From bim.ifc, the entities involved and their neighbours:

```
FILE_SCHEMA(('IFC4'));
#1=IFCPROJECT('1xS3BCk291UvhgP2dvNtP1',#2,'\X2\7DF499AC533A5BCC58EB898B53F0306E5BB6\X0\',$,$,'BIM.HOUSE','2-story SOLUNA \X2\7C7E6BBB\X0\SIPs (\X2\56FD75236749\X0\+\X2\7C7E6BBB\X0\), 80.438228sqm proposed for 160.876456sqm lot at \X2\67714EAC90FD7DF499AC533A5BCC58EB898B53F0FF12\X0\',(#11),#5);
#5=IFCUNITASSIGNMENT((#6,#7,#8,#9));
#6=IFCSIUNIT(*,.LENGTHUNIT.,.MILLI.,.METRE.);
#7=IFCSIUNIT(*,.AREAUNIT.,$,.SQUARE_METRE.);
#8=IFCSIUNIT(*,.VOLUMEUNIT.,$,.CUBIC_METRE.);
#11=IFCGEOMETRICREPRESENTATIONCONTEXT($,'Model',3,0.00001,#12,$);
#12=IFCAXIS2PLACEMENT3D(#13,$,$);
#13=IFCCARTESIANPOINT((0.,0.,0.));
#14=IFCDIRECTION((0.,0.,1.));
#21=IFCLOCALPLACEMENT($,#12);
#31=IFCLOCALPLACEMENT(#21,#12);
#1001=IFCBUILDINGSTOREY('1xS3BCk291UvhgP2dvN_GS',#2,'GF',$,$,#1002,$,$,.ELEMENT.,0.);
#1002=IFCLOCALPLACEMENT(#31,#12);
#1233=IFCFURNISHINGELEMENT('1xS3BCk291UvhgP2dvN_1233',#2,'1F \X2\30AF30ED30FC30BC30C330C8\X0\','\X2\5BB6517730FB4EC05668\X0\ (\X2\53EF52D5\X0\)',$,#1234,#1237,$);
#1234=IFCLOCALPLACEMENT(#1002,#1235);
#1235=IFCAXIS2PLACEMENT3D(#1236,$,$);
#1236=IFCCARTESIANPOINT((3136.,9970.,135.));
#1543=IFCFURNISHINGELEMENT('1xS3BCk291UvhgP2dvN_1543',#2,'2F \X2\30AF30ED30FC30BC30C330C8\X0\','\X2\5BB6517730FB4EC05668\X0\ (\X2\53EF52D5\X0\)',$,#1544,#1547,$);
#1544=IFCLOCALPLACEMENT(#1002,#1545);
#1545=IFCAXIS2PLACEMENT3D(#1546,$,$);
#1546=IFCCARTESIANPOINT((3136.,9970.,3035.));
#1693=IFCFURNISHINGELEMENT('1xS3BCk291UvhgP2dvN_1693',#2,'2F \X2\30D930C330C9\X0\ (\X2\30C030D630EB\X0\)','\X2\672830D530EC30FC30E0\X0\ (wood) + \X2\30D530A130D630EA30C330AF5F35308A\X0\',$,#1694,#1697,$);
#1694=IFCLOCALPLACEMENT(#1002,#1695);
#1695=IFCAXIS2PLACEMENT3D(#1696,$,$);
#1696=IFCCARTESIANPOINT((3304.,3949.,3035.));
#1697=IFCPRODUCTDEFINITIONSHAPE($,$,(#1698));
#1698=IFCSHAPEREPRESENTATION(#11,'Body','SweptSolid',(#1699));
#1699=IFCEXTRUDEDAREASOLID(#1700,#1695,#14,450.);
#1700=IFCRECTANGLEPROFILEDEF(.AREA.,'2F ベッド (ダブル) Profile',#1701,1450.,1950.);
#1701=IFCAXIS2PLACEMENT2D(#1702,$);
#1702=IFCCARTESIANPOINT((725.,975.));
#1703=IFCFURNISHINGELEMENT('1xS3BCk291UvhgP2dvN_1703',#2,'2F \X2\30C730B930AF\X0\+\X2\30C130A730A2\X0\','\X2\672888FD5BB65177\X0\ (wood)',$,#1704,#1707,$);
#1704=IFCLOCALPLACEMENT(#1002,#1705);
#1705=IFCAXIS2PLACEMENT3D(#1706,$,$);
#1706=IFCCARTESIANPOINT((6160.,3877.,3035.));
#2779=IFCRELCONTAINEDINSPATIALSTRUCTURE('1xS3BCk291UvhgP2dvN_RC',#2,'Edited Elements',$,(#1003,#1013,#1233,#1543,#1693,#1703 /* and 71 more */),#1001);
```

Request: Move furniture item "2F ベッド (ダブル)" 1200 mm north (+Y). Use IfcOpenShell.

```python
import ifcopenshell
import ifcopenshell.api.geometry
import ifcopenshell.util.placement

model = ifcopenshell.open("bim.ifc")

item = model.by_id(1693)
matrix = ifcopenshell.util.placement.get_local_placement(item.ObjectPlacement)
matrix[1, 3] += 1200.0
ifcopenshell.api.geometry.edit_object_placement(model, product=item, matrix=matrix, is_si=False)

print(ifcopenshell.util.placement.get_local_placement(item.ObjectPlacement).round(3) + 0.0)

model.write("bim_rev.ifc")
```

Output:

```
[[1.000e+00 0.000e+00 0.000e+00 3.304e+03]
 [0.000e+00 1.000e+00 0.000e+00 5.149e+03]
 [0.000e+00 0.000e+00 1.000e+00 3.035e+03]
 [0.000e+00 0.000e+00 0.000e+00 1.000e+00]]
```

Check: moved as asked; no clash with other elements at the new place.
